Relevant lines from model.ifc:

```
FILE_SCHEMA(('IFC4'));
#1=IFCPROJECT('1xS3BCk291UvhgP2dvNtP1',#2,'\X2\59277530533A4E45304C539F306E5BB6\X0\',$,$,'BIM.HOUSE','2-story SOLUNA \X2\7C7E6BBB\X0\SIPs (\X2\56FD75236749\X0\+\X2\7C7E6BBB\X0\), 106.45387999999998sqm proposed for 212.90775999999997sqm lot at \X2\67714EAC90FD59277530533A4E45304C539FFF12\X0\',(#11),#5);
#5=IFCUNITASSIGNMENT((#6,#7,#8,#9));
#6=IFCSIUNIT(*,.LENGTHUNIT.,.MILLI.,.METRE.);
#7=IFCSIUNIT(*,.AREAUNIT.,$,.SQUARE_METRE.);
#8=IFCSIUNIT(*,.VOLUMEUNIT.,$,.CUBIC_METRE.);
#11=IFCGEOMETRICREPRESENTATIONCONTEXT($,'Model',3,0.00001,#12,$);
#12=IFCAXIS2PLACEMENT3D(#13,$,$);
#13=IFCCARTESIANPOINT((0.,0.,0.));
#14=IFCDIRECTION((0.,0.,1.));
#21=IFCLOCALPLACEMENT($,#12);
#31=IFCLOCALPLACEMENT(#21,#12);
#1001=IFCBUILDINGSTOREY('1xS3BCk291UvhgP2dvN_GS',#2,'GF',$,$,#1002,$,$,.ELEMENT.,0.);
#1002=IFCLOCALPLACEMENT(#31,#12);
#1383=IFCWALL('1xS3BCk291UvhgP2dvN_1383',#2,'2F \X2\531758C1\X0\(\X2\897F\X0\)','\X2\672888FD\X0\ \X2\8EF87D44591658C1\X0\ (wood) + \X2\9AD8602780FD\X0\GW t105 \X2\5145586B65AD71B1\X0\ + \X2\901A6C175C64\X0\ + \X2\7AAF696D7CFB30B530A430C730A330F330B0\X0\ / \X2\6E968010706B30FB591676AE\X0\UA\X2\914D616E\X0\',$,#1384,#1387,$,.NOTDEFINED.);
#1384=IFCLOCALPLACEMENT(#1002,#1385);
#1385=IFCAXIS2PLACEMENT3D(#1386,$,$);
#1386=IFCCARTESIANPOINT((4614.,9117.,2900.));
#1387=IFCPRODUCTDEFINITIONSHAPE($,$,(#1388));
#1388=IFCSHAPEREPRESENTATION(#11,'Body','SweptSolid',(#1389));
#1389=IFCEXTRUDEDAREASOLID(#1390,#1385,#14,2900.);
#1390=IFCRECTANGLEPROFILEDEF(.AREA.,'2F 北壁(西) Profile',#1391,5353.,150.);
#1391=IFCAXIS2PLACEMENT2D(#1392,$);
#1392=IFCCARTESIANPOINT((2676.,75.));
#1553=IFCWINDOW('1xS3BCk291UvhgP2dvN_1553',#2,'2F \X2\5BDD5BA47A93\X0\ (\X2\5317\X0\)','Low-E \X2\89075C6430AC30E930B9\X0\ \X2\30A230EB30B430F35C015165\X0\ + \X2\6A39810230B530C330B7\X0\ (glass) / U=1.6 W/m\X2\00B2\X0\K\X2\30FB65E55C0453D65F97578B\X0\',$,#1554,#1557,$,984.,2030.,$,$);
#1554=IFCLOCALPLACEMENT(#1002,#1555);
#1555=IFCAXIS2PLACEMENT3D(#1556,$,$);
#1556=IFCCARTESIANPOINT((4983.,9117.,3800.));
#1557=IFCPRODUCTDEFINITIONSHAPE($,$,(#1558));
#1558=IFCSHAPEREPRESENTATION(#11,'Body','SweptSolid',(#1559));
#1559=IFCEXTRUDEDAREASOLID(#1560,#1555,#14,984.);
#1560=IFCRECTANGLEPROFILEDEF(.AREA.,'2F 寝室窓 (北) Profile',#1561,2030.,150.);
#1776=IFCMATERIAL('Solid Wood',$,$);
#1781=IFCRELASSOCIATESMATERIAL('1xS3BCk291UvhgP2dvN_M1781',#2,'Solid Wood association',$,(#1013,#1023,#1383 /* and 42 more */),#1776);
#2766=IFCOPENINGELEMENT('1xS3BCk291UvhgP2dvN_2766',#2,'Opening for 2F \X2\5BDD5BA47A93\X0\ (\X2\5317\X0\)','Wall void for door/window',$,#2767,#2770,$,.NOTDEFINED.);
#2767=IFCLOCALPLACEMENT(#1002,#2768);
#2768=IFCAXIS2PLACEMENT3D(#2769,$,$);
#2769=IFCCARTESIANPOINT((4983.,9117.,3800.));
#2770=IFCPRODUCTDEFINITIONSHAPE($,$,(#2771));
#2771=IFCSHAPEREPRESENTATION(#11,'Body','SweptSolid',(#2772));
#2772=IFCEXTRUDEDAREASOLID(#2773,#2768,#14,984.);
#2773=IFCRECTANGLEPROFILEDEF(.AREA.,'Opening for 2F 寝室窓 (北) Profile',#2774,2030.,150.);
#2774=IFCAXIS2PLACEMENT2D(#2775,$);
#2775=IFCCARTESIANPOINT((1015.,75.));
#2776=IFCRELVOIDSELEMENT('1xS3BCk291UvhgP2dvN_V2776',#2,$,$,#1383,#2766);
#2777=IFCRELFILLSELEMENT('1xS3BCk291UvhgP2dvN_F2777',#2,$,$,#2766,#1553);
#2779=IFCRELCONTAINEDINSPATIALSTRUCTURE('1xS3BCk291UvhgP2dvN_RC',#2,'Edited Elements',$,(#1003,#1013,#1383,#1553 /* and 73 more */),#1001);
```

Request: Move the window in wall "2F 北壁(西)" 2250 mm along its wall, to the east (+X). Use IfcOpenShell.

```python
import ifcopenshell
import ifcopenshell.api.geometry
import ifcopenshell.util.placement
import ifcopenshell.util.unit

model = ifcopenshell.open("model.ifc")
unit_scale = ifcopenshell.util.unit.calculate_unit_scale(model)

window = model.by_guid("1xS3BCk291UvhgP2dvN_1553")
opening = window.FillsVoids[0].RelatingOpeningElement
wall = opening.VoidsElements[0].RelatingBuildingElement

wall_matrix = ifcopenshell.util.placement.get_local_placement(wall.ObjectPlacement)
shift = wall_matrix[:3, 0] * 2.25 / unit_scale
before = ifcopenshell.util.placement.get_local_placement(window.ObjectPlacement)[:3, 3].copy()

# The window is not placed relative to its opening, so move both.
for product in (opening, window):
    matrix = ifcopenshell.util.placement.get_local_placement(product.ObjectPlacement)
    matrix[:3, 3] += shift
    ifcopenshell.api.geometry.edit_object_placement(model, product=product, matrix=matrix, is_si=False)

after = ifcopenshell.util.placement.get_local_placement(window.ObjectPlacement)[:3, 3]
print("window moved by", (after - before).round(3) + 0.0)

model.write("model-out.ifc")
```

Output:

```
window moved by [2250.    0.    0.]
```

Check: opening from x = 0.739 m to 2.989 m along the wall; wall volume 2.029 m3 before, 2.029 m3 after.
